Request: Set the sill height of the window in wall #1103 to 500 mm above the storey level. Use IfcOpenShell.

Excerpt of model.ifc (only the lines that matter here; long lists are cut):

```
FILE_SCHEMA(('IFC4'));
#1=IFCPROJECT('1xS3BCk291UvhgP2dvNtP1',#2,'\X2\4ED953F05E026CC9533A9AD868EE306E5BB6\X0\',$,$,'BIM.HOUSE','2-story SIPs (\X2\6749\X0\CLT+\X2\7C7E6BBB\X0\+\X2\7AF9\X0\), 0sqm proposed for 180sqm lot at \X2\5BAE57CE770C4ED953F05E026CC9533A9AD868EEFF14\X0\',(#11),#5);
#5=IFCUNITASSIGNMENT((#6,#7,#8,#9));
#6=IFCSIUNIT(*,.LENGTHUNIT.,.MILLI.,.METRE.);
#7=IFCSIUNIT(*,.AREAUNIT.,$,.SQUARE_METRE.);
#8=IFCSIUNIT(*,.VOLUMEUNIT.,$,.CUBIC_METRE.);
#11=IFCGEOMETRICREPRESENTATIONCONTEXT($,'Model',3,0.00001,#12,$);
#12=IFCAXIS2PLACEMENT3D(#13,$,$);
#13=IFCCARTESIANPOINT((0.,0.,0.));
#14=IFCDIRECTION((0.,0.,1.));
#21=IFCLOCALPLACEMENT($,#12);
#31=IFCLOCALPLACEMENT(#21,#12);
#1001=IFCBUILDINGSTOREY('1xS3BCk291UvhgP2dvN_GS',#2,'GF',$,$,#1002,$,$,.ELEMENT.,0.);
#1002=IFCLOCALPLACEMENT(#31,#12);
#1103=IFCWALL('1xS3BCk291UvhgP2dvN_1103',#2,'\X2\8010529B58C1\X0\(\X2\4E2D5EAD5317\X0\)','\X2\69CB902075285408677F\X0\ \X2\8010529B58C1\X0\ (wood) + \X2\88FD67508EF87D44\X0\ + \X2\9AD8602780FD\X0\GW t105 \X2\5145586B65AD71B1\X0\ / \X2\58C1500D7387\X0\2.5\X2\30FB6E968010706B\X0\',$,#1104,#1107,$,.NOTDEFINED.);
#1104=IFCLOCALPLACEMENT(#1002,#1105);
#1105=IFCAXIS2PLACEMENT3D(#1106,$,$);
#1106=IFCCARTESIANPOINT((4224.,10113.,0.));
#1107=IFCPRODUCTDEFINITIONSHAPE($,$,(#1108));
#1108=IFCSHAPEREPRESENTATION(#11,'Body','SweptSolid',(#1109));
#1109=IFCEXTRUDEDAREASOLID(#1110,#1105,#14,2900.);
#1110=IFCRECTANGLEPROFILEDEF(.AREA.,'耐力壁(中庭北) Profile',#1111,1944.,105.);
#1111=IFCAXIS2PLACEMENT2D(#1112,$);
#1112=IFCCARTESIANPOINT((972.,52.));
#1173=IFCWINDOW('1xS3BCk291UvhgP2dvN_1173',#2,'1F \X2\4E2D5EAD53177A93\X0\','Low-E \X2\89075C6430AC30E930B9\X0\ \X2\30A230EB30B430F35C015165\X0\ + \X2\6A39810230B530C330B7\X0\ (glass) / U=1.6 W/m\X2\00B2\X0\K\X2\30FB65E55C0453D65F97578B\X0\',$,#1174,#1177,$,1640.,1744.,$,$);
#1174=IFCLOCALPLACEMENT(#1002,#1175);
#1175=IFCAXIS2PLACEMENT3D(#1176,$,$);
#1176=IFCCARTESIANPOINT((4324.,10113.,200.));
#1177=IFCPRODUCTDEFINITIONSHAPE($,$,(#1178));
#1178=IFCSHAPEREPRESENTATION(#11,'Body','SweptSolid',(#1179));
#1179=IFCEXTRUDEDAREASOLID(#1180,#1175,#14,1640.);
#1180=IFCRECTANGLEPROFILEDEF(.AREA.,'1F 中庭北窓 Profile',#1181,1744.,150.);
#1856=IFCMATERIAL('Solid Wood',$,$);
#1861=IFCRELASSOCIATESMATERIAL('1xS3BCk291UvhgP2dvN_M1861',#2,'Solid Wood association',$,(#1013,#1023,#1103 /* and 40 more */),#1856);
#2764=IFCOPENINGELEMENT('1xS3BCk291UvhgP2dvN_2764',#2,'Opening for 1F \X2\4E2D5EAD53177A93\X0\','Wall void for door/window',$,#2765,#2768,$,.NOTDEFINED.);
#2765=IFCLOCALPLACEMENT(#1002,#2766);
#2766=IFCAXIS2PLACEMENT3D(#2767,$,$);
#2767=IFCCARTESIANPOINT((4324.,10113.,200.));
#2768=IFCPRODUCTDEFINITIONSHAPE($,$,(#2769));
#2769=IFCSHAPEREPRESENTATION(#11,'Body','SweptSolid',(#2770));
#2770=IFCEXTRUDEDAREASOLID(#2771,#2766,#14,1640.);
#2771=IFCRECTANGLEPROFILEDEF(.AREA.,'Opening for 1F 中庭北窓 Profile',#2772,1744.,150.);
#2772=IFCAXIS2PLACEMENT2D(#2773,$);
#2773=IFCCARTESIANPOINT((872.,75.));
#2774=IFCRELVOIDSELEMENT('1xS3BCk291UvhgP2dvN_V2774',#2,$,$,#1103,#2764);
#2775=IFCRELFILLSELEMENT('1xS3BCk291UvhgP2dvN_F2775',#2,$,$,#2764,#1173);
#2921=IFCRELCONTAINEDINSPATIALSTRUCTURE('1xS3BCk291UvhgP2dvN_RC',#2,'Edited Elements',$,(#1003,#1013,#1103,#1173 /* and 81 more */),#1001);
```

```python
import numpy as np
import ifcopenshell
import ifcopenshell.api.geometry
import ifcopenshell.geom
import ifcopenshell.util.element
import ifcopenshell.util.placement
import ifcopenshell.util.shape
import ifcopenshell.util.unit

model = ifcopenshell.open("model.ifc")
unit_scale = ifcopenshell.util.unit.calculate_unit_scale(model)

window = model.by_id(1173)
opening = window.FillsVoids[0].RelatingOpeningElement
storey = ifcopenshell.util.element.get_container(window, ifc_class="IfcBuildingStorey")
level = ifcopenshell.util.placement.get_local_placement(storey.ObjectPlacement)[2, 3]

# The opening's origin need not be at the sill, so measure its lowest point.
shape = ifcopenshell.geom.create_shape(ifcopenshell.geom.settings(), opening)
bottom = ifcopenshell.util.shape.get_shape_bottom_elevation(shape, shape.geometry) / unit_scale
dz = level + 0.5 / unit_scale - bottom

shift = np.array([0.0, 0.0, dz])
# The window is not placed relative to its opening, so move both.
for product in (opening, window):
    matrix = ifcopenshell.util.placement.get_local_placement(product.ObjectPlacement)
    matrix[:3, 3] += shift
    ifcopenshell.api.geometry.edit_object_placement(model, product=product, matrix=matrix, is_si=False)

print(f"moved by {dz * unit_scale:+.3f} m")

model.write("model_v2.ifc")
```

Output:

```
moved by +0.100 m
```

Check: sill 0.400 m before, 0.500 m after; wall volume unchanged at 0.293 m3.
